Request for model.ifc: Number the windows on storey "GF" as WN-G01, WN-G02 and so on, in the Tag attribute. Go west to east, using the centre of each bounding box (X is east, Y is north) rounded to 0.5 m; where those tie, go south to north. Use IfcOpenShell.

First a look at what the model holds.

```python
import ifcopenshell
import ifcopenshell.util.element
import ifcopenshell.util.placement

model = ifcopenshell.open("model.ifc")
print(model.schema)
storey = next(s for s in model.by_type("IfcBuildingStorey") if s.Name == "GF")
windows = [e for e in ifcopenshell.util.element.get_decomposition(storey) if e.is_a("IfcWindow")]
for e in sorted(windows, key=lambda e: e.id()):
    origin = ifcopenshell.util.placement.get_local_placement(e.ObjectPlacement)[:3, 3]
    print(e.id(), e.Tag, e.Name, origin.round(2) + 0.0, sep=" | ")
```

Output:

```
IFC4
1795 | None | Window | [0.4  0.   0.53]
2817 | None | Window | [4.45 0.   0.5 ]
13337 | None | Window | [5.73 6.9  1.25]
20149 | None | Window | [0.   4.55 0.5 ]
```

```python
import ifcopenshell
import ifcopenshell.geom
import ifcopenshell.util.element
import ifcopenshell.util.shape

model = ifcopenshell.open("model.ifc")
settings = ifcopenshell.geom.settings()
settings.set("use-world-coords", True)


def centre(element):
    shape = ifcopenshell.geom.create_shape(settings, element)
    return ifcopenshell.util.shape.get_bbox_centroid(shape.geometry)


storey = next(s for s in model.by_type("IfcBuildingStorey") if s.Name == "GF")
windows = [e for e in ifcopenshell.util.element.get_decomposition(storey) if e.is_a("IfcWindow")]

# Insertion points can sit at a corner or the storey origin, so sort by the geometry (in metres).
centres = {e: centre(e) for e in windows}
windows.sort(key=lambda e: (round(centres[e][0] / 0.5), centres[e][1]))

for i, e in enumerate(windows, start=1):
    number = f"WN-G{i:02d}"
    e.Tag = number
    print(e.id(), number)

model.write("model_edited.ifc")
```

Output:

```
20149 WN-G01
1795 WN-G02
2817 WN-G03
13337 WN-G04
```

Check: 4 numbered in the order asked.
